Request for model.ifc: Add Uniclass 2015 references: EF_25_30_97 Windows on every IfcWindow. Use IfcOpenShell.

First a look at what the model holds.

```python
import ifcopenshell

model = ifcopenshell.open("model.ifc")
print(model.schema)
print("classifications:", [c.Name for c in model.by_type("IfcClassification")])
for ifc_class in ("IfcDoor", "IfcRoof", "IfcStair", "IfcWall", "IfcWindow"):
    print(ifc_class, len(model.by_type(ifc_class)))
```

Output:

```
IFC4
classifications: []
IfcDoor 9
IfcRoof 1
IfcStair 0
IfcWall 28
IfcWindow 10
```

```python
import ifcopenshell
import ifcopenshell.api.classification

model = ifcopenshell.open("model.ifc")

system = ifcopenshell.api.classification.add_classification(model, classification="Uniclass 2015")

codes = {
    "IfcWindow": ("EF_25_30_97", "Windows"),
}
for ifc_class, (code, name) in codes.items():
    products = model.by_type(ifc_class)
    ifcopenshell.api.classification.add_reference(
        model, products=products, classification=system, identification=code, name=name
    )
    print(code, len(products))

model.write("model_v2.ifc")
```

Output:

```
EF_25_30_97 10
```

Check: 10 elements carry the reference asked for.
